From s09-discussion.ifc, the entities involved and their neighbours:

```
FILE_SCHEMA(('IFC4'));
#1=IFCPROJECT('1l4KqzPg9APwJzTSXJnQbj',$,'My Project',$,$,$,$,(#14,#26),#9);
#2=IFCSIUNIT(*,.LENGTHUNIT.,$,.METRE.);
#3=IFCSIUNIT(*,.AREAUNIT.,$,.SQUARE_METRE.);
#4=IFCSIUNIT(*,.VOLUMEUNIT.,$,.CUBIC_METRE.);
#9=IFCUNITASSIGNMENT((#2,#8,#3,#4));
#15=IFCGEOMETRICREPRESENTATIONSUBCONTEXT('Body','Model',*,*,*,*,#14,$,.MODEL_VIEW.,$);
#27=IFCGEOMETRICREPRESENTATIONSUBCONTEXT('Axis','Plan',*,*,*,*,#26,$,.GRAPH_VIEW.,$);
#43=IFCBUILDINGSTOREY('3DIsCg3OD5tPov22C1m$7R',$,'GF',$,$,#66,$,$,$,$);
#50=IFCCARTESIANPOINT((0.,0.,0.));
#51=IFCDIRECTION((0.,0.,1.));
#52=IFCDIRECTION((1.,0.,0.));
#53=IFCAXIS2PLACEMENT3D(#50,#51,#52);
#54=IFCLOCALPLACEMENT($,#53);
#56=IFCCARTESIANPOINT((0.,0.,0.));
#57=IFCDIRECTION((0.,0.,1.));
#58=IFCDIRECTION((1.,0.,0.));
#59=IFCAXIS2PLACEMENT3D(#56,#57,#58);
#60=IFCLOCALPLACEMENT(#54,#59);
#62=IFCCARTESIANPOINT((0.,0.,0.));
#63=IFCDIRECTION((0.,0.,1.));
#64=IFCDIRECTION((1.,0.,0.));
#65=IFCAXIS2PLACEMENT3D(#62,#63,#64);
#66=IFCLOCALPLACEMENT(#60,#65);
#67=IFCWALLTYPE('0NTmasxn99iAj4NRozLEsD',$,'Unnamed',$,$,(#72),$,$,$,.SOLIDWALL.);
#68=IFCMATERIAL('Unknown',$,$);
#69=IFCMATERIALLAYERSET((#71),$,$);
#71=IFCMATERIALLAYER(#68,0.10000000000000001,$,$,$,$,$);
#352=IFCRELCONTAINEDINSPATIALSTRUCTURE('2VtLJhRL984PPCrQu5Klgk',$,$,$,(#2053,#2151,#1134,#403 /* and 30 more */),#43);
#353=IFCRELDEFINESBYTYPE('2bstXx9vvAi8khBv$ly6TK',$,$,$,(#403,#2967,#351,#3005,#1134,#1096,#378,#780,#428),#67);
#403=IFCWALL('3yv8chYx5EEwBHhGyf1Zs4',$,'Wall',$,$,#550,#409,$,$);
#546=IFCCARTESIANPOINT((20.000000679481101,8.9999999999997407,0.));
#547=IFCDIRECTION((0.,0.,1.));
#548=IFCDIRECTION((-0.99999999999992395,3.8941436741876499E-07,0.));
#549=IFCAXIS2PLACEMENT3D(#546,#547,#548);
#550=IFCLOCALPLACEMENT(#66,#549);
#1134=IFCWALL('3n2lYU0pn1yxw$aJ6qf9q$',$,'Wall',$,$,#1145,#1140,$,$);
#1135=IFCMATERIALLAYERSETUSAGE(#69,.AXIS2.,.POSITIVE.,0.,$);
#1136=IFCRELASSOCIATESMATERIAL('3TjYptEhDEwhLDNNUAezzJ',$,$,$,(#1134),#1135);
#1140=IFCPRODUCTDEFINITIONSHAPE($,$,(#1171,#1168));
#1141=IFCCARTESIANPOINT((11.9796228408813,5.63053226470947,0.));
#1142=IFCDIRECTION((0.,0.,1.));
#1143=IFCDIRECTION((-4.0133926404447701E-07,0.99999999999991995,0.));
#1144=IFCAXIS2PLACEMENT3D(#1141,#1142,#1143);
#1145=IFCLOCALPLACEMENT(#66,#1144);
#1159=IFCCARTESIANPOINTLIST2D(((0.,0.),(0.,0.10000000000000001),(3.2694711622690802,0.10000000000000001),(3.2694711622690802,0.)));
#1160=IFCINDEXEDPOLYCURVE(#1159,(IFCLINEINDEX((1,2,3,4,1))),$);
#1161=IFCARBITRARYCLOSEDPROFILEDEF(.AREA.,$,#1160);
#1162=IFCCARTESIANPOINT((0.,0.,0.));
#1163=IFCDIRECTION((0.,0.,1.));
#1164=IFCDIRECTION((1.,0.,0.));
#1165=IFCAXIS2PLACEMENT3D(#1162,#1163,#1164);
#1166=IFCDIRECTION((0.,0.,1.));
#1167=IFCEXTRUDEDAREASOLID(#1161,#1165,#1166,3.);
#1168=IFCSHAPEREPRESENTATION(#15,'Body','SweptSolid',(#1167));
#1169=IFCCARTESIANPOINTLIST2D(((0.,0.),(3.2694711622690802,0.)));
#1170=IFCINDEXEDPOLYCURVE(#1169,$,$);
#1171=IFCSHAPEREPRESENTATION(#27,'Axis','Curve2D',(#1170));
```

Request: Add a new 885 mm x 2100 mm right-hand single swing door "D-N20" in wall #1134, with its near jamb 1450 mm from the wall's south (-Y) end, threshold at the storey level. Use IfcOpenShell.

```python
import numpy as np
import ifcopenshell
import ifcopenshell.api.feature
import ifcopenshell.api.geometry
import ifcopenshell.api.root
import ifcopenshell.api.spatial
import ifcopenshell.geom
import ifcopenshell.util.element
import ifcopenshell.util.placement
import ifcopenshell.util.representation
import ifcopenshell.util.shape
import ifcopenshell.util.unit

model = ifcopenshell.open("s09-discussion.ifc")
unit_scale = ifcopenshell.util.unit.calculate_unit_scale(model)
settings = ifcopenshell.geom.settings()


def volume(element):
    """Net volume in cubic metres, openings subtracted."""
    shape = ifcopenshell.geom.create_shape(settings, element)
    return ifcopenshell.util.shape.get_volume(shape.geometry)


wall = model.by_guid("3n2lYU0pn1yxw$aJ6qf9q$")
storey = ifcopenshell.util.element.get_container(wall, ifc_class="IfcBuildingStorey")
context = ifcopenshell.util.representation.get_context(model, "Model", "Body", "MODEL_VIEW")
before = volume(wall)

width, height, from_end, sill = 0.885, 2.1, 1.45, 0.0  # metres

# The wall runs along its own X axis, and the end named is its -X end.
wall_shape = ifcopenshell.geom.create_shape(settings, wall)
x, y, z = ifcopenshell.util.shape.get_vertices(wall_shape.geometry).T
start = x.min() + from_end
face, thickness = float(y.min()), float(y.max() - y.min())
wall_matrix = ifcopenshell.util.placement.get_local_placement(wall.ObjectPlacement)
level = ifcopenshell.util.placement.get_local_placement(storey.ObjectPlacement)[2, 3]


def in_wall(x, y):
    """Placement at x, y metres in the wall's axes, at sill height."""
    matrix = wall_matrix.copy()
    matrix[:, 3] = wall_matrix @ np.array([x / unit_scale, y / unit_scale, 0.0, 1.0])
    matrix[2, 3] = level + sill / unit_scale
    return matrix


# Opening: a box that overshoots both wall faces by 50 mm.
opening = ifcopenshell.api.root.create_entity(model, ifc_class="IfcOpeningElement", predefined_type="OPENING")
box = ifcopenshell.api.geometry.add_wall_representation(
    model, context=context, length=width, height=height, thickness=thickness + 0.1
)
ifcopenshell.api.geometry.assign_representation(model, product=opening, representation=box)
ifcopenshell.api.geometry.edit_object_placement(model, product=opening, matrix=in_wall(start, face - 0.05), is_si=False)
ifcopenshell.api.feature.add_feature(model, feature=opening, element=wall)

door = ifcopenshell.api.root.create_entity(model, ifc_class="IfcDoor", name="D-N20", predefined_type="DOOR")
door.OverallWidth, door.OverallHeight = width / unit_scale, height / unit_scale
door.OperationType = "SINGLE_SWING_RIGHT"
body = ifcopenshell.api.geometry.add_door_representation(
    model,
    context=context,
    overall_width=door.OverallWidth,
    overall_height=door.OverallHeight,
    operation_type="SINGLE_SWING_RIGHT",
    lining_properties={"LiningDepth": thickness / unit_scale, "ThresholdDepth": thickness / unit_scale},
)
ifcopenshell.api.geometry.assign_representation(model, product=door, representation=body)
ifcopenshell.api.spatial.assign_container(model, products=[door], relating_structure=storey)
ifcopenshell.api.feature.add_filling(model, opening=opening, element=door)

# The lining spans the wall, so the door starts at the wall face.
ifcopenshell.api.geometry.edit_object_placement(model, product=door, matrix=in_wall(start, face), is_si=False)

after = volume(wall)

print(f"wall volume {before:.3f} -> {after:.3f} m3")

model.write("s09-discussion_updated.ifc")
```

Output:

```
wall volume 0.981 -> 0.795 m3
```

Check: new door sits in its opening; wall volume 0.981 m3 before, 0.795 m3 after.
